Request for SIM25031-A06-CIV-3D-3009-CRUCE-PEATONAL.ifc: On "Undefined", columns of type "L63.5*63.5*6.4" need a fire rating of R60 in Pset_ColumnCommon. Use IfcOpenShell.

First a look at what the model holds.

```python
import ifcopenshell
import ifcopenshell.util.element

model = ifcopenshell.open("SIM25031-A06-CIV-3D-3009-CRUCE-PEATONAL.ifc")
print(model.schema)
storey = next(s for s in model.by_type("IfcBuildingStorey") if s.Name == "Undefined")
columns = [e for e in ifcopenshell.util.element.get_decomposition(storey) if e.is_a("IfcColumn")]
seen = {}
for e in columns:
    element_type = ifcopenshell.util.element.get_type(e)
    key = (element_type.Name if element_type != e and element_type else None, ifcopenshell.util.element.get_pset(e, "Pset_ColumnCommon", "FireRating"))
    seen[key] = seen.get(key, 0) + 1
for (name, value), count in sorted(seen.items(), key=str):
    print(count, "x", name, "|", value)
```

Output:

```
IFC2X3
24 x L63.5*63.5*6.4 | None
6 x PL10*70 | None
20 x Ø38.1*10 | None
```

```python
import ifcopenshell
import ifcopenshell.api.pset
import ifcopenshell.util.element

model = ifcopenshell.open("SIM25031-A06-CIV-3D-3009-CRUCE-PEATONAL.ifc")

storey = next(s for s in model.by_type("IfcBuildingStorey") if s.Name == "Undefined")
columns = [e for e in ifcopenshell.util.element.get_decomposition(storey) if e.is_a("IfcColumn")]

count = 0
for e in columns:
    element_type = ifcopenshell.util.element.get_type(e)
    if element_type in (None, e) or element_type.Name != "L63.5*63.5*6.4":
        continue
    found = ifcopenshell.util.element.get_pset(e, "Pset_ColumnCommon", should_inherit=False)
    if found:
        pset = model.by_id(found["id"])
        if len(ifcopenshell.util.element.get_elements_by_pset(pset)) > 1:
            pset = ifcopenshell.api.pset.unshare_pset(model, products=[e], pset=pset)[0]
    else:
        pset = ifcopenshell.api.pset.add_pset(model, product=e, name="Pset_ColumnCommon")
    ifcopenshell.api.pset.edit_pset(model, pset=pset, properties={"FireRating": "R60"})
    count += 1

print(count, "columns updated")

model.write("SIM25031-A06-CIV-3D-3009-CRUCE-PEATONAL_edited.ifc")
```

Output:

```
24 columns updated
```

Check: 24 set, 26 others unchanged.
